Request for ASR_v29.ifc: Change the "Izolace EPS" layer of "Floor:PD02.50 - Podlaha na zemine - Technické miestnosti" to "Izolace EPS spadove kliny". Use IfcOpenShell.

First a look at what the model holds.

```python
import ifcopenshell
import ifcopenshell.util.element

model = ifcopenshell.open("ASR_v29.ifc")
print(model.schema)
for layer_set in model.by_type("IfcMaterialLayerSet"):
    if layer_set.LayerSetName == "Floor:PD02.50 - Podlaha na zemine - Technické miestnosti":
        for layer in layer_set.MaterialLayers:
            print(layer.id(), layer.Material and layer.Material.Name, layer.LayerThickness, sep=" | ")
        print(len(ifcopenshell.util.element.get_elements_by_material(model, layer_set)), "elements and types use it")
print(sorted(m.Name for m in model.by_type("IfcMaterial") if m.Name)[:60])
```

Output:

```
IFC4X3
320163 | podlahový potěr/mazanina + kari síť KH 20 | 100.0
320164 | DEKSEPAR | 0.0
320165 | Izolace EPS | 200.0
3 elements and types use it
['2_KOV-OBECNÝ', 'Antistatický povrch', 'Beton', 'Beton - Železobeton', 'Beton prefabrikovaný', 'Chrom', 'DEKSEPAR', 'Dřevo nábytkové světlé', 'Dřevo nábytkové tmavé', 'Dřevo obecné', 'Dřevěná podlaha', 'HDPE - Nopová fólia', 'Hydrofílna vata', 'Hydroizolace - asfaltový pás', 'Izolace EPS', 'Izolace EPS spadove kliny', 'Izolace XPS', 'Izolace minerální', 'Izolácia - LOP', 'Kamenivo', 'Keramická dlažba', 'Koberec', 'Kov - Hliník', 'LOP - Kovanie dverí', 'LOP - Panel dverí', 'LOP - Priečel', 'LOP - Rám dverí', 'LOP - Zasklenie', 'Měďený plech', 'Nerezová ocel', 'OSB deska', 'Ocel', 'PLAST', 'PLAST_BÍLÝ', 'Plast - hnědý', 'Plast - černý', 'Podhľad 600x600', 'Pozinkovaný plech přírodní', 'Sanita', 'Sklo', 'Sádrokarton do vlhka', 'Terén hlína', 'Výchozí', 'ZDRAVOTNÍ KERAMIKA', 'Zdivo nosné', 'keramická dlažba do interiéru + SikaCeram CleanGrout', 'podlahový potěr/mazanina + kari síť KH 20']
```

```python
import ifcopenshell
import ifcopenshell.api.material

model = ifcopenshell.open("ASR_v29.ifc")

layer_set = next(s for s in model.by_type("IfcMaterialLayerSet") if s.LayerSetName == "Floor:PD02.50 - Podlaha na zemine - Technické miestnosti")
layer = next(l for l in layer_set.MaterialLayers if l.Material and l.Material.Name == "Izolace EPS")
material = next(m for m in model.by_type("IfcMaterial") if m.Name == "Izolace EPS spadove kliny")

# Point this one layer at the other material; renaming the old one would change it everywhere.
ifcopenshell.api.material.edit_layer(model, layer=layer, attributes={"Name": material.Name}, material=material)

print([l.Material.Name if l.Material else None for l in layer_set.MaterialLayers])

model.write("ASR_v29-out.ifc")
```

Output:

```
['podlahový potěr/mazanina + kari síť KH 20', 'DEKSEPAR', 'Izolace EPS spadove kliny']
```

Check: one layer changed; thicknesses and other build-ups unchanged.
